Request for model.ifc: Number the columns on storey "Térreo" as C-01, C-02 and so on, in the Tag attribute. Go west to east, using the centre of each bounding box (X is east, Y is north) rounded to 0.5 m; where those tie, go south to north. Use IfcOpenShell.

First a look at what the model holds.

```python
import ifcopenshell
import ifcopenshell.util.element
import ifcopenshell.util.placement

model = ifcopenshell.open("model.ifc")
print(model.schema)
storey = next(s for s in model.by_type("IfcBuildingStorey") if s.Name == "Térreo")
columns = [e for e in ifcopenshell.util.element.get_decomposition(storey) if e.is_a("IfcColumn")]
for e in sorted(columns, key=lambda e: e.id()):
    origin = ifcopenshell.util.placement.get_local_placement(e.ObjectPlacement)[:3, 3]
    print(e.id(), e.Tag, e.Name, origin.round(2) + 0.0, sep=" | ")
```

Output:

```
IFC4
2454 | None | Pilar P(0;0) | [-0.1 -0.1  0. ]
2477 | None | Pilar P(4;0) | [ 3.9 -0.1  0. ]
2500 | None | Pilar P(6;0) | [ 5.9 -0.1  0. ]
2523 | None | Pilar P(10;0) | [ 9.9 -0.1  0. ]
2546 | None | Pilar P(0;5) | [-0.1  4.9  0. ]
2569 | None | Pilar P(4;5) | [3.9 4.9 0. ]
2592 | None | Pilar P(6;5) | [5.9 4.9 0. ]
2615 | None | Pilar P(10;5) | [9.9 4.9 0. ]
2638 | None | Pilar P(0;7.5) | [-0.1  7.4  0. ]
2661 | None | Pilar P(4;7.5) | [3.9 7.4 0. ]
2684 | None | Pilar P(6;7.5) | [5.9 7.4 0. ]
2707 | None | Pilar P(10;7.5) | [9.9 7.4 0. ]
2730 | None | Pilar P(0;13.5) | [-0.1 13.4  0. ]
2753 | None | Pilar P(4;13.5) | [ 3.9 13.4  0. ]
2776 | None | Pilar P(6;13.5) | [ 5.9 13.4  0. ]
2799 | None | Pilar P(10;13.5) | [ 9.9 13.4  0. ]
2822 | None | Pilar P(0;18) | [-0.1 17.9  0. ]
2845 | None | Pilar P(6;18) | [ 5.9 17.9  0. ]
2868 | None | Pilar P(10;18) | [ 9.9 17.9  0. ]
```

```python
import ifcopenshell
import ifcopenshell.geom
import ifcopenshell.util.element
import ifcopenshell.util.shape

model = ifcopenshell.open("model.ifc")
settings = ifcopenshell.geom.settings()
settings.set("use-world-coords", True)


def centre(element):
    shape = ifcopenshell.geom.create_shape(settings, element)
    return ifcopenshell.util.shape.get_bbox_centroid(shape.geometry)


storey = next(s for s in model.by_type("IfcBuildingStorey") if s.Name == "Térreo")
columns = [e for e in ifcopenshell.util.element.get_decomposition(storey) if e.is_a("IfcColumn")]

# Insertion points can sit at a corner or the storey origin, so sort by the geometry (in metres).
centres = {e: centre(e) for e in columns}
columns.sort(key=lambda e: (round(centres[e][0] / 0.5), centres[e][1]))

for i, e in enumerate(columns, start=1):
    number = f"C-{i:02d}"
    e.Tag = number
    print(e.id(), number)

model.write("model_rev.ifc")
```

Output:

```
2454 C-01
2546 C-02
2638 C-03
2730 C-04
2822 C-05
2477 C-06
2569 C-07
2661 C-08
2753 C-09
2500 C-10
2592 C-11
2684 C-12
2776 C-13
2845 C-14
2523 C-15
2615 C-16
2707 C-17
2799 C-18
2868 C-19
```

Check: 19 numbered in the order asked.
